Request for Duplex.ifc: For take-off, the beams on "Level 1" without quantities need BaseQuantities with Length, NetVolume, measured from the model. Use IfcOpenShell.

First a look at what the model holds.

```python
import ifcopenshell
import ifcopenshell.util.element
import ifcopenshell.util.unit

model = ifcopenshell.open("Duplex.ifc")
print(model.schema)
for unit_type in ("LENGTHUNIT", "AREAUNIT", "VOLUMEUNIT"):
    print(unit_type, ifcopenshell.util.unit.calculate_unit_scale(model, unit_type))
storey = next(s for s in model.by_type("IfcBuildingStorey") if s.Name == "Level 1")
beams = [e for e in ifcopenshell.util.element.get_decomposition(storey) if e.is_a("IfcBeam")]
for e in sorted(beams, key=lambda e: e.id()):
    print(e.id(), e.is_a(), e.Name, list(ifcopenshell.util.element.get_psets(e, qtos_only=True)), sep=" | ")
```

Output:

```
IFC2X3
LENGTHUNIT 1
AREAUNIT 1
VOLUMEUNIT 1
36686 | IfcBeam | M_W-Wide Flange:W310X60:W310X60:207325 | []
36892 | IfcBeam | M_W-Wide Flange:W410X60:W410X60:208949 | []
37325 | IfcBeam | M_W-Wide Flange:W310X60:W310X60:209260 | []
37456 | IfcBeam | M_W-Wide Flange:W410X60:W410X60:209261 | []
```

```python
import ifcopenshell
import ifcopenshell.api.pset
import ifcopenshell.geom
import ifcopenshell.util.element
import ifcopenshell.util.shape
import ifcopenshell.util.unit

model = ifcopenshell.open("Duplex.ifc")
unit_scale = ifcopenshell.util.unit.calculate_unit_scale(model)
volume_scale = ifcopenshell.util.unit.calculate_unit_scale(model, "VOLUMEUNIT")
settings = ifcopenshell.geom.settings()

storey = next(s for s in model.by_type("IfcBuildingStorey") if s.Name == "Level 1")
beams = [e for e in ifcopenshell.util.element.get_decomposition(storey) if e.is_a("IfcBeam")]

for e in sorted(beams, key=lambda e: e.id()):
    if ifcopenshell.util.element.get_psets(e, qtos_only=True, should_inherit=False):
        continue
    # Geometry comes back in metres, in the element's own axes.
    shape = ifcopenshell.geom.create_shape(settings, e)
    values = {
        "Length": ifcopenshell.util.shape.get_max_xyz(shape.geometry) / unit_scale,
        "NetVolume": ifcopenshell.util.shape.get_volume(shape.geometry) / volume_scale,
    }
    qto = ifcopenshell.api.pset.add_qto(model, product=e, name="BaseQuantities")
    ifcopenshell.api.pset.edit_qto(model, qto=qto, properties=values)
    print(e.id(), {k: round(v, 3) for k, v in values.items()})

model.write("Duplex_edited.ifc")
```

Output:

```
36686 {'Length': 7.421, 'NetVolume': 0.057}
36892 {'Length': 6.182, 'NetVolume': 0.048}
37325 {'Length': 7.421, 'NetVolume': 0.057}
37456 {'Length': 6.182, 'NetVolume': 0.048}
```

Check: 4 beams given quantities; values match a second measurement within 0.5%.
